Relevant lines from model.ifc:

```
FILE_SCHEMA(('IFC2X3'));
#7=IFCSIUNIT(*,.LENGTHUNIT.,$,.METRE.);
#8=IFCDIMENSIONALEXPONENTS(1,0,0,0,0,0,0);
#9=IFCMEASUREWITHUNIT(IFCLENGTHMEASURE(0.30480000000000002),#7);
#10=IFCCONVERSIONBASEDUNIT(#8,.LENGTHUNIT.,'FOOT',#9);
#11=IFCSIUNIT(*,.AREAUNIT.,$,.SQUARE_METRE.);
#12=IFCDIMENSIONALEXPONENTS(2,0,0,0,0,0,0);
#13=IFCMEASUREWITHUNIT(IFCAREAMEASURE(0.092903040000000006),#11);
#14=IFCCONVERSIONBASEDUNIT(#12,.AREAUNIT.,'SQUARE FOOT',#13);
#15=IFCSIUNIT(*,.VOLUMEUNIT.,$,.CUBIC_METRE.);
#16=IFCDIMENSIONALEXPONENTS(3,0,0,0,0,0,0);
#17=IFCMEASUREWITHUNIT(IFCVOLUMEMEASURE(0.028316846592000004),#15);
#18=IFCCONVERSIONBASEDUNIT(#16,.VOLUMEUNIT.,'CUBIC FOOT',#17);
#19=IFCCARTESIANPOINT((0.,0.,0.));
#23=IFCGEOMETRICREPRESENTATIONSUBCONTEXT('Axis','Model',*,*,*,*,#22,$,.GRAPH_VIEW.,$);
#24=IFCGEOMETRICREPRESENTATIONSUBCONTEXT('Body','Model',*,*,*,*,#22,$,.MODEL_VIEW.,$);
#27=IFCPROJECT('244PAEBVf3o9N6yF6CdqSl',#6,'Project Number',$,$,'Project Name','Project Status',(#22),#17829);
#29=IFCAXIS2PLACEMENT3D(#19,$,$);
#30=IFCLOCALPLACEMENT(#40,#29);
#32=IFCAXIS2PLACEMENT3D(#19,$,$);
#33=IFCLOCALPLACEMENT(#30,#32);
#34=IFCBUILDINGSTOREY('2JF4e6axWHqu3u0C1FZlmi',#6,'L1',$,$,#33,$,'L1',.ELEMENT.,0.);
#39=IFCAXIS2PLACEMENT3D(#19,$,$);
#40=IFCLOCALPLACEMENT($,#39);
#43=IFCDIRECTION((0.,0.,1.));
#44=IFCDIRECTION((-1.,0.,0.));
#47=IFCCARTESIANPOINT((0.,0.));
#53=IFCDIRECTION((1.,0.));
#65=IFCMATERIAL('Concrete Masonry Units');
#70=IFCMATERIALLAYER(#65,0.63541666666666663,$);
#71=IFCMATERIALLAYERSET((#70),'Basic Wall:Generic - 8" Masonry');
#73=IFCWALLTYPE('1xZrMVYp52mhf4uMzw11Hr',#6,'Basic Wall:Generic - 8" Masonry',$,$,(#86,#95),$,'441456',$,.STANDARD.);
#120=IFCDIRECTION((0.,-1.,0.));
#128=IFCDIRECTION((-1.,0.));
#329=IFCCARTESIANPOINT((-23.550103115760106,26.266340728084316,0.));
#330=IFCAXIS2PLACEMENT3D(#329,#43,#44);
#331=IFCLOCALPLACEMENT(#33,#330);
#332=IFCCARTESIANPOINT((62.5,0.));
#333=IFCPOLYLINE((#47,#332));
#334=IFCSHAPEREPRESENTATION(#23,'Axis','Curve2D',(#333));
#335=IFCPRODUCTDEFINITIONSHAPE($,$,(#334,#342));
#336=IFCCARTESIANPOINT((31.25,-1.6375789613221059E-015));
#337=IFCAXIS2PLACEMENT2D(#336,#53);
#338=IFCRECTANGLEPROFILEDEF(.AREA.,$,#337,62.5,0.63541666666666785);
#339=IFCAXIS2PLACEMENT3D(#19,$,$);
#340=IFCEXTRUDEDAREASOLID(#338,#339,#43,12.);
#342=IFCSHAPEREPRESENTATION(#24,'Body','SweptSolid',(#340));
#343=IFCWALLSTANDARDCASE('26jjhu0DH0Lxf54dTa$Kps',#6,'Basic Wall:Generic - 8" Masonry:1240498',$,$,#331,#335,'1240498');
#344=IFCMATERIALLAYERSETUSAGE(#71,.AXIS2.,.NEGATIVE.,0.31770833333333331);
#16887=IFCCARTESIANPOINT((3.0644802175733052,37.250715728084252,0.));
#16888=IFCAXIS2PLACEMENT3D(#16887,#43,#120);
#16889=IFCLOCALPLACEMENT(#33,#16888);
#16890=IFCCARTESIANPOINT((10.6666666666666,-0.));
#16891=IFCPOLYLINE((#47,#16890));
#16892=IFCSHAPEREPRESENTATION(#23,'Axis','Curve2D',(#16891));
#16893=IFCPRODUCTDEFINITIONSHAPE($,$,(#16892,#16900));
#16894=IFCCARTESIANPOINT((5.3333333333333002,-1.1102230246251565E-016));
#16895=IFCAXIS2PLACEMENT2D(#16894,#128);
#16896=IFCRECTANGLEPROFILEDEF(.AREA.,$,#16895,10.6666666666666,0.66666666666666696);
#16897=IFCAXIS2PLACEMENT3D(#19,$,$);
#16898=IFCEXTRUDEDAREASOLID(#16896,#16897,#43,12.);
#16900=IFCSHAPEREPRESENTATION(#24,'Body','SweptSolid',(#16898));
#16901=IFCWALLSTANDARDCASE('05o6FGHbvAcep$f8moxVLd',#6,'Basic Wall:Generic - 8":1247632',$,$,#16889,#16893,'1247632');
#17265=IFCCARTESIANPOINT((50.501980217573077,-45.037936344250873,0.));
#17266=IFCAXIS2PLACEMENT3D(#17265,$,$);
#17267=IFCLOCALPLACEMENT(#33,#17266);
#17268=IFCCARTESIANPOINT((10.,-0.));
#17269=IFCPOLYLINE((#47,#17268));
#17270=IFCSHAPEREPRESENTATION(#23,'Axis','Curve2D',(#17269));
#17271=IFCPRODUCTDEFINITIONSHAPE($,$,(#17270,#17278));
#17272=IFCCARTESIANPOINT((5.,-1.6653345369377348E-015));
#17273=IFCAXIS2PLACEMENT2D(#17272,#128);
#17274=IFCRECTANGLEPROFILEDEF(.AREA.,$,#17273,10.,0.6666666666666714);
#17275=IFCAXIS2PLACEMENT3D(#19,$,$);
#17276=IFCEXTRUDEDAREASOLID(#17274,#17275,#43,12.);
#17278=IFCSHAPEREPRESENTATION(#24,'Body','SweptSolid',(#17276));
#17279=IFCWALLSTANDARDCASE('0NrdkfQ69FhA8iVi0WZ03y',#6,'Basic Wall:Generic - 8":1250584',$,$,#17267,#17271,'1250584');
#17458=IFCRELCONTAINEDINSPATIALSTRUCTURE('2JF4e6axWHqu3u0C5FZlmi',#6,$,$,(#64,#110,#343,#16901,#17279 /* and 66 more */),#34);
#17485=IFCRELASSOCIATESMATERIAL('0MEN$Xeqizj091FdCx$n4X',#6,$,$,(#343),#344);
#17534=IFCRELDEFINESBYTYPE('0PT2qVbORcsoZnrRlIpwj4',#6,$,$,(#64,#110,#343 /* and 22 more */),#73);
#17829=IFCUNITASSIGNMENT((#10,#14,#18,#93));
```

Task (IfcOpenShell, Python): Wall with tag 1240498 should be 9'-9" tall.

```python
import ifcopenshell
import ifcopenshell.geom
import ifcopenshell.util.representation
import ifcopenshell.util.shape
import ifcopenshell.util.unit

model = ifcopenshell.open("model.ifc")
unit_scale = ifcopenshell.util.unit.calculate_unit_scale(model)
settings = ifcopenshell.geom.settings()


def volume(element):
    """Net volume in cubic metres, openings subtracted."""
    shape = ifcopenshell.geom.create_shape(settings, element)
    return ifcopenshell.util.shape.get_volume(shape.geometry)


wall = model.by_id(343)
before = volume(wall)

body = ifcopenshell.util.representation.get_representation(wall, "Model", "Body")
solid = body.Items[0]
old_height = solid.Depth
solid.Depth = 117 * 0.0254 / unit_scale
after = volume(wall)

print(f"height {old_height:g} -> {solid.Depth:g}, volume {before:.3f} -> {after:.3f} m3")

model.write("model_rev.ifc")
```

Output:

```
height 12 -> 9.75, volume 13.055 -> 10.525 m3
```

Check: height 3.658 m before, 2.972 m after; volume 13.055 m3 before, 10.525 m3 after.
